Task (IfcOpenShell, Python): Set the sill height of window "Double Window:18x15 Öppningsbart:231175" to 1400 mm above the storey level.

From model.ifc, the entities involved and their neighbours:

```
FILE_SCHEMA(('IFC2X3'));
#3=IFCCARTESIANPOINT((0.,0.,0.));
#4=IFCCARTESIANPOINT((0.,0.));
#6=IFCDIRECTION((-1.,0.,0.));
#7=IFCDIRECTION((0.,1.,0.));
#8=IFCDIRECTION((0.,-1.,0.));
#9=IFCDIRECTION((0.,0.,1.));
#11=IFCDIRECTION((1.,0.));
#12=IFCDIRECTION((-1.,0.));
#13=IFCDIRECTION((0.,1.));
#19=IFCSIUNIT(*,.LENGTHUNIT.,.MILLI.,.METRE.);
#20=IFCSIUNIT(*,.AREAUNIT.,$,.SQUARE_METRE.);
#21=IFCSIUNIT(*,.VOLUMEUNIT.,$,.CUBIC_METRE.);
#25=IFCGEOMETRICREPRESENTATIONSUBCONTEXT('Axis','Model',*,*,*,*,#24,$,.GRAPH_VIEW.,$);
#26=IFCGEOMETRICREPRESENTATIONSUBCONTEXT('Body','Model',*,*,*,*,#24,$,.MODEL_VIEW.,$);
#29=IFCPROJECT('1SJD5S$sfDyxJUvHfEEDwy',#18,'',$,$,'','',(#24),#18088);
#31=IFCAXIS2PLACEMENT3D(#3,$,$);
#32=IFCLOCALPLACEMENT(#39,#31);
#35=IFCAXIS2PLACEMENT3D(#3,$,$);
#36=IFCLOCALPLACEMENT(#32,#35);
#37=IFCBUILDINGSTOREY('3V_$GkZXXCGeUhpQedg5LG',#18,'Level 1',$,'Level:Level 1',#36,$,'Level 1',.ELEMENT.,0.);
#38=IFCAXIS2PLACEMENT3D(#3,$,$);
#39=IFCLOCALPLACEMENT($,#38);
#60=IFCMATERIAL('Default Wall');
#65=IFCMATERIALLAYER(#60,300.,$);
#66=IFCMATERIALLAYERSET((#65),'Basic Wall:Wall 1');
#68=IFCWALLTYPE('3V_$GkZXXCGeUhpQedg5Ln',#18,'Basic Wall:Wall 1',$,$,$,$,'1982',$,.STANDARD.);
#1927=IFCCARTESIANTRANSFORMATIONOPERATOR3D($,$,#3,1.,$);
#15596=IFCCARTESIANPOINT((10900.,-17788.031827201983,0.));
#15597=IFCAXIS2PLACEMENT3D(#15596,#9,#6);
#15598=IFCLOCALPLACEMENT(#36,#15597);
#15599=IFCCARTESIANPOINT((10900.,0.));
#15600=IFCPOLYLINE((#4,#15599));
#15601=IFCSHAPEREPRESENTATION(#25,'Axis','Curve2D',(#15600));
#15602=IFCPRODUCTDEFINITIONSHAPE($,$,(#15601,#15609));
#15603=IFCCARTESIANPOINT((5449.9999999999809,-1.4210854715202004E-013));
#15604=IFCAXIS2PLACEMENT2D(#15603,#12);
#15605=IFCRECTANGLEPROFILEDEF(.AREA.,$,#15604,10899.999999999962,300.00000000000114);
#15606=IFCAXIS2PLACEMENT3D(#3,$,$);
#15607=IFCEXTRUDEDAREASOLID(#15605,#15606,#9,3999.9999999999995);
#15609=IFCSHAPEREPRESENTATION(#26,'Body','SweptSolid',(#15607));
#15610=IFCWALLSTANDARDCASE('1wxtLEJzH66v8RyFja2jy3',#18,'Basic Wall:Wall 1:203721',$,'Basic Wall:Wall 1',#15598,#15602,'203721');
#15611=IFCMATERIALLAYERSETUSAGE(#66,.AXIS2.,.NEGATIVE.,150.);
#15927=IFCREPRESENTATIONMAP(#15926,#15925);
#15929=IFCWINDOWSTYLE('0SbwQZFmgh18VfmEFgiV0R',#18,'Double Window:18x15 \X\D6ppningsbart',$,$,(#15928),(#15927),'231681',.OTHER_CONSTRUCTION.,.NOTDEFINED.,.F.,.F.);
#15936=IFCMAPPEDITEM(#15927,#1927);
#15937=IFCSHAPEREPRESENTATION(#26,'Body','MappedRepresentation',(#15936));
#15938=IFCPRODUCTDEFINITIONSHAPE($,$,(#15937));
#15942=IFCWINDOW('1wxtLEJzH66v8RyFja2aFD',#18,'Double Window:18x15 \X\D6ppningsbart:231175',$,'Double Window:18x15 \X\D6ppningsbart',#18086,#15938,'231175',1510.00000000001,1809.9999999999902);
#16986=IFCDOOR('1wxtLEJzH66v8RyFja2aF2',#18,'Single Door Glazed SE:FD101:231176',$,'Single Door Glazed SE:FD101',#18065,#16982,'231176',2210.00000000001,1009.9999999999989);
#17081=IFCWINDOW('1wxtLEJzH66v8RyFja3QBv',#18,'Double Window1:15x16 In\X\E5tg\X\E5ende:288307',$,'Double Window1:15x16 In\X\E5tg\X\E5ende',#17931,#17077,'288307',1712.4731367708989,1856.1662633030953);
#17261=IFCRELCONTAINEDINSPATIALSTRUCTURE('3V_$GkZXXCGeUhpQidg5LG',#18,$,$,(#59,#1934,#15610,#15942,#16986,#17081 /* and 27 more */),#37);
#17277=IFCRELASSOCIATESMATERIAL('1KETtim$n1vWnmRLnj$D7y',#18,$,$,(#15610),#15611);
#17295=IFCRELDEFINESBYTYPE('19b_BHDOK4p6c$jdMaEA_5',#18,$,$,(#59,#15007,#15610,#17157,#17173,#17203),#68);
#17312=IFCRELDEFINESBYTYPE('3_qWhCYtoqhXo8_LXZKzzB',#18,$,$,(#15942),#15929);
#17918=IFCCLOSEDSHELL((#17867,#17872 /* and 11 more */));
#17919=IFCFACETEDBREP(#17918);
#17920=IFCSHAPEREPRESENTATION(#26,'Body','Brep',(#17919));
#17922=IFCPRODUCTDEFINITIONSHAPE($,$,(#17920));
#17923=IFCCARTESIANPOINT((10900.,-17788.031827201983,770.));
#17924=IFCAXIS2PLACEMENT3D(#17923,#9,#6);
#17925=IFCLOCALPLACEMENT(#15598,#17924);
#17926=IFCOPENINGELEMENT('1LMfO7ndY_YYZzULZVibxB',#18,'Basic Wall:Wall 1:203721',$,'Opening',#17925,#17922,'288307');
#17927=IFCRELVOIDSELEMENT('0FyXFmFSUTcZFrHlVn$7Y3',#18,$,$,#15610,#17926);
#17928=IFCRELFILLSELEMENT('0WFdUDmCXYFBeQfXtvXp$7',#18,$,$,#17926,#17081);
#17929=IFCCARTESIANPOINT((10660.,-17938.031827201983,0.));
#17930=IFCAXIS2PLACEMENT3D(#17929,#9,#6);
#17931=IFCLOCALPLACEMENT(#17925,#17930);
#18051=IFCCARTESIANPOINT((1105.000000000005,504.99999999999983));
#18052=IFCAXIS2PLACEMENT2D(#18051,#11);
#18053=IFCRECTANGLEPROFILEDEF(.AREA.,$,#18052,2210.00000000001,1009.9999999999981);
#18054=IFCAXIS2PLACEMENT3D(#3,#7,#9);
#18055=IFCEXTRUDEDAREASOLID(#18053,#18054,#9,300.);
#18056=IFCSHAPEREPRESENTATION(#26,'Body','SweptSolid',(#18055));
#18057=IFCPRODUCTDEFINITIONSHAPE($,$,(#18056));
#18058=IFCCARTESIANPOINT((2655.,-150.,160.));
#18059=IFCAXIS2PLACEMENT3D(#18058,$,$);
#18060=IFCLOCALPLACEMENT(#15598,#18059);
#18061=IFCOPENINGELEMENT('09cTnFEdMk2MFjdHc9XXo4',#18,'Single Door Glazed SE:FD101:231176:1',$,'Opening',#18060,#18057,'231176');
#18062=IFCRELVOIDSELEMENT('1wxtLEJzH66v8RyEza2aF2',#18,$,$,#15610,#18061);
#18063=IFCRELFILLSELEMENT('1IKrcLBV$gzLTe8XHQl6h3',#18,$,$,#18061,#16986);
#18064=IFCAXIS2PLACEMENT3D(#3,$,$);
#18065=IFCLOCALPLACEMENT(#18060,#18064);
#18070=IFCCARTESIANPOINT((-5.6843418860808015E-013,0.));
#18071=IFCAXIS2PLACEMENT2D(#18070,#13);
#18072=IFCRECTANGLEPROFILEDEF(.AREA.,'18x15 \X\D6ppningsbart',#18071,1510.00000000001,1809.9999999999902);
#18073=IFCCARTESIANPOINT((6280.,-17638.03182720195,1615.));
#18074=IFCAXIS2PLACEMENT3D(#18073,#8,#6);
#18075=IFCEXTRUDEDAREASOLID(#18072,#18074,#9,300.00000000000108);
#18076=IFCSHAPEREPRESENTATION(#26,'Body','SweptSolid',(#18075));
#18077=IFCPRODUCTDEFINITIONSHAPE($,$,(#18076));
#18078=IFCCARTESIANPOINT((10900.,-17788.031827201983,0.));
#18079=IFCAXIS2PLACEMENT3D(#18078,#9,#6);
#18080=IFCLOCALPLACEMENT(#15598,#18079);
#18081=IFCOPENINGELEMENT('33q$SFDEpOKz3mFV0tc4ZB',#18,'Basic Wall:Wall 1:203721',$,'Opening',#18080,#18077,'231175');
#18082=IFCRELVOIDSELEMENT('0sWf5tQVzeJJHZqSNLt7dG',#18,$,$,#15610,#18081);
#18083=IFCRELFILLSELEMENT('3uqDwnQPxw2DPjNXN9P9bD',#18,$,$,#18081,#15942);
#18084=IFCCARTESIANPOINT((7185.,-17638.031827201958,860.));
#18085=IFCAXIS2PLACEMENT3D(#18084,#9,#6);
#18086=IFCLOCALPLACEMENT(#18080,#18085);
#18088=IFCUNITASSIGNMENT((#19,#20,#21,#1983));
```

```python
import numpy as np
import ifcopenshell
import ifcopenshell.api.geometry
import ifcopenshell.geom
import ifcopenshell.util.element
import ifcopenshell.util.placement
import ifcopenshell.util.shape
import ifcopenshell.util.unit

model = ifcopenshell.open("model.ifc")
unit_scale = ifcopenshell.util.unit.calculate_unit_scale(model)

window = model.by_id(15942)
opening = window.FillsVoids[0].RelatingOpeningElement
storey = ifcopenshell.util.element.get_container(window, ifc_class="IfcBuildingStorey")
level = ifcopenshell.util.placement.get_local_placement(storey.ObjectPlacement)[2, 3]

# The opening's origin need not be at the sill, so measure its lowest point.
shape = ifcopenshell.geom.create_shape(ifcopenshell.geom.settings(), opening)
bottom = ifcopenshell.util.shape.get_shape_bottom_elevation(shape, shape.geometry) / unit_scale
dz = level + 1.4 / unit_scale - bottom

shift = np.array([0.0, 0.0, dz])
# The window is placed relative to its opening, so it follows when the opening moves.
matrix = ifcopenshell.util.placement.get_local_placement(opening.ObjectPlacement)
matrix[:3, 3] += shift
ifcopenshell.api.geometry.edit_object_placement(
    model, product=opening, matrix=matrix, is_si=False, should_transform_children=True
)

print(f"moved by {dz * unit_scale:+.3f} m")

model.write("model_rev.ifc")
```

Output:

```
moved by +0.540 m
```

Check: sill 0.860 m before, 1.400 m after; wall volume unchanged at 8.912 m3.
